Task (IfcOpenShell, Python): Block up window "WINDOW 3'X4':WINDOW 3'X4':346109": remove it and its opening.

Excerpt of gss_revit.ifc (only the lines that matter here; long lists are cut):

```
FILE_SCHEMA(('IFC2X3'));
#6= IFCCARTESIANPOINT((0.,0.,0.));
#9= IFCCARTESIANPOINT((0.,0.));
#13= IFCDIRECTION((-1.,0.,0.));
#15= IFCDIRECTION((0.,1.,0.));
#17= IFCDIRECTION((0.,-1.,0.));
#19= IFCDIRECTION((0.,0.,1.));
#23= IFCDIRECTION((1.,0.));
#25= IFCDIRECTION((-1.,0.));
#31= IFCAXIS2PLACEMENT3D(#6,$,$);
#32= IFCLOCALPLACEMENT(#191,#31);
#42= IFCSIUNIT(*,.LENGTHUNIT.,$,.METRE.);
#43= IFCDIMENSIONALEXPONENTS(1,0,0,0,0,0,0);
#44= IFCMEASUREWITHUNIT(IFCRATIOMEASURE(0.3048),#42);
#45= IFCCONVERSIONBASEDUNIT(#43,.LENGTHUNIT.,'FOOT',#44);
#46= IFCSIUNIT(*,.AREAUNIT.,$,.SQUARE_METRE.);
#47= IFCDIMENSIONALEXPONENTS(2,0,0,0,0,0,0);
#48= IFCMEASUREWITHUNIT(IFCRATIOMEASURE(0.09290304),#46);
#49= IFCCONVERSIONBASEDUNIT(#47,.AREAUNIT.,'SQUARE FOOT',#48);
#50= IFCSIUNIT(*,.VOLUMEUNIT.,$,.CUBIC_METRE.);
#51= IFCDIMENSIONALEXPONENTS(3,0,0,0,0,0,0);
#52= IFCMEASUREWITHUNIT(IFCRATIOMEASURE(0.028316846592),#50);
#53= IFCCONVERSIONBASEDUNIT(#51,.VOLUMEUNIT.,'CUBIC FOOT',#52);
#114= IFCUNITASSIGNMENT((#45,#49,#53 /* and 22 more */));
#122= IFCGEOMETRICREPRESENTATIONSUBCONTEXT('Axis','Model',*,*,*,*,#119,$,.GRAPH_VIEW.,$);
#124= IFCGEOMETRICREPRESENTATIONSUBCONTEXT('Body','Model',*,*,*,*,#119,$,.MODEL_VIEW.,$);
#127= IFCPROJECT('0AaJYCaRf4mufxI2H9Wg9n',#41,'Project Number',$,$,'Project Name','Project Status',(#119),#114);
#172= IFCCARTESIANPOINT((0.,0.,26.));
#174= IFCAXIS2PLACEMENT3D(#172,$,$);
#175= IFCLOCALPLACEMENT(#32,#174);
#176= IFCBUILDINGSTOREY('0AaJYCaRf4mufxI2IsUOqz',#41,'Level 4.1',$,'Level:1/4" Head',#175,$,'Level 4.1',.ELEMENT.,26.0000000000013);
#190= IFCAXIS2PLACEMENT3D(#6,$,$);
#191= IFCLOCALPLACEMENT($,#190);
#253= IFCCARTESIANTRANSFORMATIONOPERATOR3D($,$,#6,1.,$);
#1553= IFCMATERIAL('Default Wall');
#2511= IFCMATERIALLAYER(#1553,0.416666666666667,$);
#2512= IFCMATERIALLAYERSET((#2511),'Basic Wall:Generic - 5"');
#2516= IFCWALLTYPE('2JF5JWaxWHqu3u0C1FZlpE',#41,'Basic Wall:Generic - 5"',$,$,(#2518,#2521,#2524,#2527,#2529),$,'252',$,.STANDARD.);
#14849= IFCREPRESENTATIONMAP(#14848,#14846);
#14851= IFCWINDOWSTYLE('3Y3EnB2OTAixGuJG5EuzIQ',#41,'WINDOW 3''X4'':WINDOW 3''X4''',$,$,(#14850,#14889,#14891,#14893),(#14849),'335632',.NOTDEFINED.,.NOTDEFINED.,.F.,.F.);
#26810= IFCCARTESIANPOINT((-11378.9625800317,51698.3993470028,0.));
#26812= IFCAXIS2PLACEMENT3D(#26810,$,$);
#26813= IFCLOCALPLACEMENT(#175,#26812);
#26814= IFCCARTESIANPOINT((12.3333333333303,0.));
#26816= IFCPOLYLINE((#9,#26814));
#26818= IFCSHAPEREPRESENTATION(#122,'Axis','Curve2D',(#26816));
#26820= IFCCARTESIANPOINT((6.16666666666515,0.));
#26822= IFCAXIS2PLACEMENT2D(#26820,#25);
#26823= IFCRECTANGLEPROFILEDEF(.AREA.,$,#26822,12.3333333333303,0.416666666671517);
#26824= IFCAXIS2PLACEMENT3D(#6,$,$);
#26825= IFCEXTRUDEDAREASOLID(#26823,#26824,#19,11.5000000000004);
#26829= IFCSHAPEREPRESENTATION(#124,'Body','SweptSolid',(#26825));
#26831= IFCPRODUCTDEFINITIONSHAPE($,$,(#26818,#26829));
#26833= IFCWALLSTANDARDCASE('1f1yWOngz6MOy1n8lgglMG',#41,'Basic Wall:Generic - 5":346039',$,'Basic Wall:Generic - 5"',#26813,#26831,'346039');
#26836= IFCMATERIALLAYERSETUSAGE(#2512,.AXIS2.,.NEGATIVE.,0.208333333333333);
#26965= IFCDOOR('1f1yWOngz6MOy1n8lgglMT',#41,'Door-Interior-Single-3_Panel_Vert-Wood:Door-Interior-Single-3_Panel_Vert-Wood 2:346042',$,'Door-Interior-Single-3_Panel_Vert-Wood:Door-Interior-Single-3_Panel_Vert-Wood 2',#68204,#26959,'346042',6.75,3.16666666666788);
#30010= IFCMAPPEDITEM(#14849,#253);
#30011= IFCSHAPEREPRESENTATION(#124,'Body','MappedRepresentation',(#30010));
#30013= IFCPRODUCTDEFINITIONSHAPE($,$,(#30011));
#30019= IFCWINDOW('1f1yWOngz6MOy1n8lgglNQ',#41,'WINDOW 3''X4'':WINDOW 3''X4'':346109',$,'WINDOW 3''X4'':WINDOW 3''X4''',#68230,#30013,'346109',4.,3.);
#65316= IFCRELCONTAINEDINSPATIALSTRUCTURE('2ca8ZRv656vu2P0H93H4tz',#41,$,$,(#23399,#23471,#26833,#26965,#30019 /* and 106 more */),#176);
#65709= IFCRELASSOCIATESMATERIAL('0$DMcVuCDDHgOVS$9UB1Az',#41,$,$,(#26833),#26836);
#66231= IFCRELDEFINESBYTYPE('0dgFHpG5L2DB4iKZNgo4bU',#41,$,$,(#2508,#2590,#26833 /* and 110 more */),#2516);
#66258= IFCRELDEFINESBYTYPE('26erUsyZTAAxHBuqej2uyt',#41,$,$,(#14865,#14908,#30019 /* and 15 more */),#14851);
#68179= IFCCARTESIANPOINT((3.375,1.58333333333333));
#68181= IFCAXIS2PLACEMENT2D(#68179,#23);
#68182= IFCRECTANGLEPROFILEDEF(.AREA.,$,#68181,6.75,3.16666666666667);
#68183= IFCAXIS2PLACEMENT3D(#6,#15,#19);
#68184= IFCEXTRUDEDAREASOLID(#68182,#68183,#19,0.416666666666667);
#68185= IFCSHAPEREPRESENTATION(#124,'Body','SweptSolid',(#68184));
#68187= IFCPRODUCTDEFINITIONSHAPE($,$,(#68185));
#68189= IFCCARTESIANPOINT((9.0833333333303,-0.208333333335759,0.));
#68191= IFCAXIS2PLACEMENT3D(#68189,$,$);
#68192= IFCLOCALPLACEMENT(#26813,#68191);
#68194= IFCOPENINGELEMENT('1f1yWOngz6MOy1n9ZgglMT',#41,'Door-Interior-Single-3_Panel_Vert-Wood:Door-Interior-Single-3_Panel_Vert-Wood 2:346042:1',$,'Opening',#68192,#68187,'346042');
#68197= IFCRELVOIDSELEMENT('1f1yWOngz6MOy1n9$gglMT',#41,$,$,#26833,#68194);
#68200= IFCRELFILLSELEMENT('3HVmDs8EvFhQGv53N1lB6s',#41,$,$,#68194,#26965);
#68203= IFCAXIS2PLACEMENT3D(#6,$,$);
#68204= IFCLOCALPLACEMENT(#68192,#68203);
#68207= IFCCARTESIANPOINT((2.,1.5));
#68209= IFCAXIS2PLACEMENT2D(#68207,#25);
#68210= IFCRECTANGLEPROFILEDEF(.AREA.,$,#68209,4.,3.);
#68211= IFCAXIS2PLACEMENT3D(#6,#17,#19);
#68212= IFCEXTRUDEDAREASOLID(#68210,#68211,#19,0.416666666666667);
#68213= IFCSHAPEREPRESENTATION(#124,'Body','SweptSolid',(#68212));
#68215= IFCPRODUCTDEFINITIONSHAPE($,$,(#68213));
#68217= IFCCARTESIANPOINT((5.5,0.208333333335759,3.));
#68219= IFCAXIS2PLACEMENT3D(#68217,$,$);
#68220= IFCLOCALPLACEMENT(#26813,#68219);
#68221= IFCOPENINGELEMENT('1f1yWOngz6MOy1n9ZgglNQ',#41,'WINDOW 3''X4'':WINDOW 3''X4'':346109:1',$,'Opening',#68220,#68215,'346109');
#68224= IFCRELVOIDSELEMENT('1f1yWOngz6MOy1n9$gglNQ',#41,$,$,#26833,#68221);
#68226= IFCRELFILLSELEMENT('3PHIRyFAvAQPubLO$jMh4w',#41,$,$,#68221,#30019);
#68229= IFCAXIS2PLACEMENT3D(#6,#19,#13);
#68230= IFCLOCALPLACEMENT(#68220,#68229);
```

```python
import ifcopenshell
import ifcopenshell.api.feature
import ifcopenshell.api.root
import ifcopenshell.geom
import ifcopenshell.util.shape

model = ifcopenshell.open("gss_revit.ifc")
settings = ifcopenshell.geom.settings()


def volume(element):
    """Net volume in cubic metres, openings subtracted."""
    shape = ifcopenshell.geom.create_shape(settings, element)
    return ifcopenshell.util.shape.get_volume(shape.geometry)


window = model.by_id(30019)
opening = window.FillsVoids[0].RelatingOpeningElement
wall = opening.VoidsElements[0].RelatingBuildingElement
before = volume(wall)

ifcopenshell.api.root.remove_product(model, product=window)
ifcopenshell.api.feature.remove_feature(model, feature=opening)

after = volume(wall)

print(f"wall volume {before:.3f} -> {after:.3f} m3")

model.write("gss_revit_updated.ifc")
```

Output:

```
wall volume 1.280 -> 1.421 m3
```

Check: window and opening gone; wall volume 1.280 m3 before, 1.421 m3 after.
